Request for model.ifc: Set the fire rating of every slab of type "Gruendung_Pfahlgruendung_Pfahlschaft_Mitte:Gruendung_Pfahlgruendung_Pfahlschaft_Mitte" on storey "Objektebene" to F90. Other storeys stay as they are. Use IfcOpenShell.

First a look at what the model holds.

```python
import ifcopenshell
import ifcopenshell.util.element

model = ifcopenshell.open("model.ifc")
print(model.schema)
storey = next(s for s in model.by_type("IfcBuildingStorey") if s.Name == "Objektebene")
slabs = [e for e in ifcopenshell.util.element.get_decomposition(storey) if e.is_a("IfcSlab")]
seen = {}
for e in slabs:
    element_type = ifcopenshell.util.element.get_type(e)
    key = (element_type.Name if element_type != e and element_type else None, ifcopenshell.util.element.get_pset(e, "Pset_SlabCommon", "FireRating"))
    seen[key] = seen.get(key, 0) + 1
for (name, value), count in sorted(seen.items(), key=str):
    print(count, "x", name, "|", value)
```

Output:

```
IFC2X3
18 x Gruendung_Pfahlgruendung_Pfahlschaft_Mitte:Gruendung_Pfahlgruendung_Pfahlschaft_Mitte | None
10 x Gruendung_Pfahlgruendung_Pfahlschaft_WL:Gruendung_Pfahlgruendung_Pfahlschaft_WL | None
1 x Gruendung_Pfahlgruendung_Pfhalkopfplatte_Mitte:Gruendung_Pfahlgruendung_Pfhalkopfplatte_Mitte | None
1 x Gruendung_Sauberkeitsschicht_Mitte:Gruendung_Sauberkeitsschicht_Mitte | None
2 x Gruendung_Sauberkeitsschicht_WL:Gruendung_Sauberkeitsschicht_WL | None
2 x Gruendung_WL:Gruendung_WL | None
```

```python
import ifcopenshell
import ifcopenshell.api.pset
import ifcopenshell.util.element

model = ifcopenshell.open("model.ifc")

storey = next(s for s in model.by_type("IfcBuildingStorey") if s.Name == "Objektebene")
slabs = [e for e in ifcopenshell.util.element.get_decomposition(storey) if e.is_a("IfcSlab")]

count = 0
for e in slabs:
    element_type = ifcopenshell.util.element.get_type(e)
    if element_type in (None, e) or element_type.Name != "Gruendung_Pfahlgruendung_Pfahlschaft_Mitte:Gruendung_Pfahlgruendung_Pfahlschaft_Mitte":
        continue
    # add_pset returns the element's existing set when there is one.
    pset = ifcopenshell.api.pset.add_pset(model, product=e, name="Pset_SlabCommon")
    ifcopenshell.api.pset.edit_pset(model, pset=pset, properties={"FireRating": "F90"})
    count += 1

print(count, "slabs updated")

model.write("model_edited.ifc")
```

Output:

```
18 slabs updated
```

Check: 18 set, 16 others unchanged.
